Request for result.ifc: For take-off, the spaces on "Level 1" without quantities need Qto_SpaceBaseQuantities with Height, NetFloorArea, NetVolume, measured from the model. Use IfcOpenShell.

First a look at what the model holds.

```python
import ifcopenshell
import ifcopenshell.util.element
import ifcopenshell.util.unit

model = ifcopenshell.open("result.ifc")
print(model.schema)
for unit_type in ("LENGTHUNIT", "AREAUNIT", "VOLUMEUNIT"):
    print(unit_type, ifcopenshell.util.unit.calculate_unit_scale(model, unit_type))
storey = next(s for s in model.by_type("IfcBuildingStorey") if s.Name == "Level 1")
spaces = [e for e in ifcopenshell.util.element.get_decomposition(storey) if e.is_a("IfcSpace")]
for e in sorted(spaces, key=lambda e: e.id()):
    print(e.id(), e.is_a(), e.Name, list(ifcopenshell.util.element.get_psets(e, qtos_only=True)), sep=" | ")
```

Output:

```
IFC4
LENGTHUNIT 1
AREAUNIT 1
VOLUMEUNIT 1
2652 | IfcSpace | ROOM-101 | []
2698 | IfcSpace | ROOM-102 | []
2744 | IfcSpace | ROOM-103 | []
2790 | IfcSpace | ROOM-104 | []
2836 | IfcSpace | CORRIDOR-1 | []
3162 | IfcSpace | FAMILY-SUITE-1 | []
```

```python
import ifcopenshell
import ifcopenshell.api.pset
import ifcopenshell.geom
import ifcopenshell.util.element
import ifcopenshell.util.shape
import ifcopenshell.util.unit

model = ifcopenshell.open("result.ifc")
unit_scale = ifcopenshell.util.unit.calculate_unit_scale(model)
area_scale = ifcopenshell.util.unit.calculate_unit_scale(model, "AREAUNIT")
volume_scale = ifcopenshell.util.unit.calculate_unit_scale(model, "VOLUMEUNIT")
settings = ifcopenshell.geom.settings()

storey = next(s for s in model.by_type("IfcBuildingStorey") if s.Name == "Level 1")
spaces = [e for e in ifcopenshell.util.element.get_decomposition(storey) if e.is_a("IfcSpace")]

for e in sorted(spaces, key=lambda e: e.id()):
    if ifcopenshell.util.element.get_psets(e, qtos_only=True, should_inherit=False):
        continue
    # Geometry comes back in metres, in the element's own axes.
    shape = ifcopenshell.geom.create_shape(settings, e)
    values = {
        "Height": ifcopenshell.util.shape.get_z(shape.geometry) / unit_scale,
        "NetFloorArea": ifcopenshell.util.shape.get_footprint_area(shape.geometry) / area_scale,
        "NetVolume": ifcopenshell.util.shape.get_volume(shape.geometry) / volume_scale,
    }
    qto = ifcopenshell.api.pset.add_qto(model, product=e, name="Qto_SpaceBaseQuantities")
    ifcopenshell.api.pset.edit_qto(model, qto=qto, properties=values)
    print(e.id(), {k: round(v, 3) for k, v in values.items()})

model.write("result_rev.ifc")
```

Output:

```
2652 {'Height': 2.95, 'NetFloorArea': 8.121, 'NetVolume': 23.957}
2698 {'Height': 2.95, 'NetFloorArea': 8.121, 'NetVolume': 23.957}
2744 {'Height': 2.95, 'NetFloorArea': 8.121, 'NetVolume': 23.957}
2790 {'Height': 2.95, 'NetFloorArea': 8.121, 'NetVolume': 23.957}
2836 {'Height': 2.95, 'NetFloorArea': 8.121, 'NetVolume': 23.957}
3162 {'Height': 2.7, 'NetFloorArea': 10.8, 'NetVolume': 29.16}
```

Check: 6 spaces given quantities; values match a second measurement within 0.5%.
